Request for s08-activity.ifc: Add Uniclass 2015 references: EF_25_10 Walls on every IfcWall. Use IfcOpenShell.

First a look at what the model holds.

```python
import ifcopenshell

model = ifcopenshell.open("s08-activity.ifc")
print(model.schema)
print("classifications:", [c.Name for c in model.by_type("IfcClassification")])
for ifc_class in ("IfcDoor", "IfcRoof", "IfcStair", "IfcWall", "IfcWindow"):
    print(ifc_class, len(model.by_type(ifc_class)))
```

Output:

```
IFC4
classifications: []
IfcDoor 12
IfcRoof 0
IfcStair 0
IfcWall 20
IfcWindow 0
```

```python
import ifcopenshell
import ifcopenshell.api.classification

model = ifcopenshell.open("s08-activity.ifc")

system = ifcopenshell.api.classification.add_classification(model, classification="Uniclass 2015")

codes = {
    "IfcWall": ("EF_25_10", "Walls"),
}
for ifc_class, (code, name) in codes.items():
    products = model.by_type(ifc_class)
    ifcopenshell.api.classification.add_reference(
        model, products=products, classification=system, identification=code, name=name
    )
    print(code, len(products))

model.write("s08-activity_v2.ifc")
```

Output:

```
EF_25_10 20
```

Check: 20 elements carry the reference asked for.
